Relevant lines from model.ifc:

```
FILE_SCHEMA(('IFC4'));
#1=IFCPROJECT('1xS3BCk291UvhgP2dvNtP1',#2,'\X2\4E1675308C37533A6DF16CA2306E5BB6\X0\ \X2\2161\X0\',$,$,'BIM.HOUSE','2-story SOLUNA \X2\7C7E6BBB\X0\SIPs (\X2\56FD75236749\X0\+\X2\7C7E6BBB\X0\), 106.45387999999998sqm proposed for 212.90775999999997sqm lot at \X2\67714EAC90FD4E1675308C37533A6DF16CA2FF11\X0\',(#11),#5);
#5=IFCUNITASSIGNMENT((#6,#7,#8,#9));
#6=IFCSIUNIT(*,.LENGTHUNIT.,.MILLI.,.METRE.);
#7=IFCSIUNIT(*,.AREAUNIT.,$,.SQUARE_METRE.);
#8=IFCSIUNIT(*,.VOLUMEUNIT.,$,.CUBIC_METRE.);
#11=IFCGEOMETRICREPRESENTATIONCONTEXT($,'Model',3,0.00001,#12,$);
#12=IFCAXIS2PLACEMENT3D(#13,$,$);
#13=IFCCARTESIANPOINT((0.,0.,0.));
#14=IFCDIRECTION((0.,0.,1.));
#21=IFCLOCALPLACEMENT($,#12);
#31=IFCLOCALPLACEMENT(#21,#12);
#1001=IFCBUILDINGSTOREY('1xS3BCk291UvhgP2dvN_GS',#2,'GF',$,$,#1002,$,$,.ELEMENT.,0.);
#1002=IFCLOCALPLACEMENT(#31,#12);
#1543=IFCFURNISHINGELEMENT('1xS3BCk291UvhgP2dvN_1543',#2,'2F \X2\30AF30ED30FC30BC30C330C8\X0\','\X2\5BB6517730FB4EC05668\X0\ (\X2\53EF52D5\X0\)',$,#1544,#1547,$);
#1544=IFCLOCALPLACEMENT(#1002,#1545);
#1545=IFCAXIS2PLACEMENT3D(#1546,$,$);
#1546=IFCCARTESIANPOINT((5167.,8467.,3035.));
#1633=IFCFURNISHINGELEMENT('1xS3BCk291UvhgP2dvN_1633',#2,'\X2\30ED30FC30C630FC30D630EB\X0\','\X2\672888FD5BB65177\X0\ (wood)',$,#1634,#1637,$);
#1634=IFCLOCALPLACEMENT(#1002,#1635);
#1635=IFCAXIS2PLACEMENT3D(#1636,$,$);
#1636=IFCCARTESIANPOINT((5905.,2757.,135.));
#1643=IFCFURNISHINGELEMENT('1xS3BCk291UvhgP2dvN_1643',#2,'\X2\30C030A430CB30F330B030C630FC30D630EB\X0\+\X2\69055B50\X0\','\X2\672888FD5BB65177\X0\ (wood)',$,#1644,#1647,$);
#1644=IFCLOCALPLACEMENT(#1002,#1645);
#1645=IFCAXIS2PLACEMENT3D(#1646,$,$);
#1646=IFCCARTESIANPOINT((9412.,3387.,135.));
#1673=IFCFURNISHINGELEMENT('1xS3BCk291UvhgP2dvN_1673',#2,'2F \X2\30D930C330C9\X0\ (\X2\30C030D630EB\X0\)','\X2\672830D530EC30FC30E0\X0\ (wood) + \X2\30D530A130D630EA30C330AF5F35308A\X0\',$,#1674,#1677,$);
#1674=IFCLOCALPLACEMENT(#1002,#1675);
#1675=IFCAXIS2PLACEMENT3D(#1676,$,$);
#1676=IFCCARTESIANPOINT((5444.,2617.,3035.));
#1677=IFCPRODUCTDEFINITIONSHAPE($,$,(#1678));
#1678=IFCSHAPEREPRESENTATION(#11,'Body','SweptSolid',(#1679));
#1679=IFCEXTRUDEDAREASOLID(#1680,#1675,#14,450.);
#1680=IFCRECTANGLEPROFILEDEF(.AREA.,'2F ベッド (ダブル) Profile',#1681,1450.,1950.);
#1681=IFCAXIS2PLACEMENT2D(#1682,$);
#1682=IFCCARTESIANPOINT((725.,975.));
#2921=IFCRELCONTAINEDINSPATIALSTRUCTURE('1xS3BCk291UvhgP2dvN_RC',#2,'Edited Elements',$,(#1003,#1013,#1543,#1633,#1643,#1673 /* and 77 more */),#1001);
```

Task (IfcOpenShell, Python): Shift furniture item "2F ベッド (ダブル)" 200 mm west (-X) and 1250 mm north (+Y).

```python
import ifcopenshell
import ifcopenshell.api.geometry
import ifcopenshell.util.placement
import ifcopenshell.util.unit

model = ifcopenshell.open("model.ifc")
unit_scale = ifcopenshell.util.unit.calculate_unit_scale(model)

item = model.by_guid("1xS3BCk291UvhgP2dvN_1673")
matrix = ifcopenshell.util.placement.get_local_placement(item.ObjectPlacement)
matrix[0, 3] -= 0.2 / unit_scale
matrix[1, 3] += 1.25 / unit_scale
ifcopenshell.api.geometry.edit_object_placement(model, product=item, matrix=matrix, is_si=False)

print(ifcopenshell.util.placement.get_local_placement(item.ObjectPlacement).round(3) + 0.0)

model.write("model_v2.ifc")
```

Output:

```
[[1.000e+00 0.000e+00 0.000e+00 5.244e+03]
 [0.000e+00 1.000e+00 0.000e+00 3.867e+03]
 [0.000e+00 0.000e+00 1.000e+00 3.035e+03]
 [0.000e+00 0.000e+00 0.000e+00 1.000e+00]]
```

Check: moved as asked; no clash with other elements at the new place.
